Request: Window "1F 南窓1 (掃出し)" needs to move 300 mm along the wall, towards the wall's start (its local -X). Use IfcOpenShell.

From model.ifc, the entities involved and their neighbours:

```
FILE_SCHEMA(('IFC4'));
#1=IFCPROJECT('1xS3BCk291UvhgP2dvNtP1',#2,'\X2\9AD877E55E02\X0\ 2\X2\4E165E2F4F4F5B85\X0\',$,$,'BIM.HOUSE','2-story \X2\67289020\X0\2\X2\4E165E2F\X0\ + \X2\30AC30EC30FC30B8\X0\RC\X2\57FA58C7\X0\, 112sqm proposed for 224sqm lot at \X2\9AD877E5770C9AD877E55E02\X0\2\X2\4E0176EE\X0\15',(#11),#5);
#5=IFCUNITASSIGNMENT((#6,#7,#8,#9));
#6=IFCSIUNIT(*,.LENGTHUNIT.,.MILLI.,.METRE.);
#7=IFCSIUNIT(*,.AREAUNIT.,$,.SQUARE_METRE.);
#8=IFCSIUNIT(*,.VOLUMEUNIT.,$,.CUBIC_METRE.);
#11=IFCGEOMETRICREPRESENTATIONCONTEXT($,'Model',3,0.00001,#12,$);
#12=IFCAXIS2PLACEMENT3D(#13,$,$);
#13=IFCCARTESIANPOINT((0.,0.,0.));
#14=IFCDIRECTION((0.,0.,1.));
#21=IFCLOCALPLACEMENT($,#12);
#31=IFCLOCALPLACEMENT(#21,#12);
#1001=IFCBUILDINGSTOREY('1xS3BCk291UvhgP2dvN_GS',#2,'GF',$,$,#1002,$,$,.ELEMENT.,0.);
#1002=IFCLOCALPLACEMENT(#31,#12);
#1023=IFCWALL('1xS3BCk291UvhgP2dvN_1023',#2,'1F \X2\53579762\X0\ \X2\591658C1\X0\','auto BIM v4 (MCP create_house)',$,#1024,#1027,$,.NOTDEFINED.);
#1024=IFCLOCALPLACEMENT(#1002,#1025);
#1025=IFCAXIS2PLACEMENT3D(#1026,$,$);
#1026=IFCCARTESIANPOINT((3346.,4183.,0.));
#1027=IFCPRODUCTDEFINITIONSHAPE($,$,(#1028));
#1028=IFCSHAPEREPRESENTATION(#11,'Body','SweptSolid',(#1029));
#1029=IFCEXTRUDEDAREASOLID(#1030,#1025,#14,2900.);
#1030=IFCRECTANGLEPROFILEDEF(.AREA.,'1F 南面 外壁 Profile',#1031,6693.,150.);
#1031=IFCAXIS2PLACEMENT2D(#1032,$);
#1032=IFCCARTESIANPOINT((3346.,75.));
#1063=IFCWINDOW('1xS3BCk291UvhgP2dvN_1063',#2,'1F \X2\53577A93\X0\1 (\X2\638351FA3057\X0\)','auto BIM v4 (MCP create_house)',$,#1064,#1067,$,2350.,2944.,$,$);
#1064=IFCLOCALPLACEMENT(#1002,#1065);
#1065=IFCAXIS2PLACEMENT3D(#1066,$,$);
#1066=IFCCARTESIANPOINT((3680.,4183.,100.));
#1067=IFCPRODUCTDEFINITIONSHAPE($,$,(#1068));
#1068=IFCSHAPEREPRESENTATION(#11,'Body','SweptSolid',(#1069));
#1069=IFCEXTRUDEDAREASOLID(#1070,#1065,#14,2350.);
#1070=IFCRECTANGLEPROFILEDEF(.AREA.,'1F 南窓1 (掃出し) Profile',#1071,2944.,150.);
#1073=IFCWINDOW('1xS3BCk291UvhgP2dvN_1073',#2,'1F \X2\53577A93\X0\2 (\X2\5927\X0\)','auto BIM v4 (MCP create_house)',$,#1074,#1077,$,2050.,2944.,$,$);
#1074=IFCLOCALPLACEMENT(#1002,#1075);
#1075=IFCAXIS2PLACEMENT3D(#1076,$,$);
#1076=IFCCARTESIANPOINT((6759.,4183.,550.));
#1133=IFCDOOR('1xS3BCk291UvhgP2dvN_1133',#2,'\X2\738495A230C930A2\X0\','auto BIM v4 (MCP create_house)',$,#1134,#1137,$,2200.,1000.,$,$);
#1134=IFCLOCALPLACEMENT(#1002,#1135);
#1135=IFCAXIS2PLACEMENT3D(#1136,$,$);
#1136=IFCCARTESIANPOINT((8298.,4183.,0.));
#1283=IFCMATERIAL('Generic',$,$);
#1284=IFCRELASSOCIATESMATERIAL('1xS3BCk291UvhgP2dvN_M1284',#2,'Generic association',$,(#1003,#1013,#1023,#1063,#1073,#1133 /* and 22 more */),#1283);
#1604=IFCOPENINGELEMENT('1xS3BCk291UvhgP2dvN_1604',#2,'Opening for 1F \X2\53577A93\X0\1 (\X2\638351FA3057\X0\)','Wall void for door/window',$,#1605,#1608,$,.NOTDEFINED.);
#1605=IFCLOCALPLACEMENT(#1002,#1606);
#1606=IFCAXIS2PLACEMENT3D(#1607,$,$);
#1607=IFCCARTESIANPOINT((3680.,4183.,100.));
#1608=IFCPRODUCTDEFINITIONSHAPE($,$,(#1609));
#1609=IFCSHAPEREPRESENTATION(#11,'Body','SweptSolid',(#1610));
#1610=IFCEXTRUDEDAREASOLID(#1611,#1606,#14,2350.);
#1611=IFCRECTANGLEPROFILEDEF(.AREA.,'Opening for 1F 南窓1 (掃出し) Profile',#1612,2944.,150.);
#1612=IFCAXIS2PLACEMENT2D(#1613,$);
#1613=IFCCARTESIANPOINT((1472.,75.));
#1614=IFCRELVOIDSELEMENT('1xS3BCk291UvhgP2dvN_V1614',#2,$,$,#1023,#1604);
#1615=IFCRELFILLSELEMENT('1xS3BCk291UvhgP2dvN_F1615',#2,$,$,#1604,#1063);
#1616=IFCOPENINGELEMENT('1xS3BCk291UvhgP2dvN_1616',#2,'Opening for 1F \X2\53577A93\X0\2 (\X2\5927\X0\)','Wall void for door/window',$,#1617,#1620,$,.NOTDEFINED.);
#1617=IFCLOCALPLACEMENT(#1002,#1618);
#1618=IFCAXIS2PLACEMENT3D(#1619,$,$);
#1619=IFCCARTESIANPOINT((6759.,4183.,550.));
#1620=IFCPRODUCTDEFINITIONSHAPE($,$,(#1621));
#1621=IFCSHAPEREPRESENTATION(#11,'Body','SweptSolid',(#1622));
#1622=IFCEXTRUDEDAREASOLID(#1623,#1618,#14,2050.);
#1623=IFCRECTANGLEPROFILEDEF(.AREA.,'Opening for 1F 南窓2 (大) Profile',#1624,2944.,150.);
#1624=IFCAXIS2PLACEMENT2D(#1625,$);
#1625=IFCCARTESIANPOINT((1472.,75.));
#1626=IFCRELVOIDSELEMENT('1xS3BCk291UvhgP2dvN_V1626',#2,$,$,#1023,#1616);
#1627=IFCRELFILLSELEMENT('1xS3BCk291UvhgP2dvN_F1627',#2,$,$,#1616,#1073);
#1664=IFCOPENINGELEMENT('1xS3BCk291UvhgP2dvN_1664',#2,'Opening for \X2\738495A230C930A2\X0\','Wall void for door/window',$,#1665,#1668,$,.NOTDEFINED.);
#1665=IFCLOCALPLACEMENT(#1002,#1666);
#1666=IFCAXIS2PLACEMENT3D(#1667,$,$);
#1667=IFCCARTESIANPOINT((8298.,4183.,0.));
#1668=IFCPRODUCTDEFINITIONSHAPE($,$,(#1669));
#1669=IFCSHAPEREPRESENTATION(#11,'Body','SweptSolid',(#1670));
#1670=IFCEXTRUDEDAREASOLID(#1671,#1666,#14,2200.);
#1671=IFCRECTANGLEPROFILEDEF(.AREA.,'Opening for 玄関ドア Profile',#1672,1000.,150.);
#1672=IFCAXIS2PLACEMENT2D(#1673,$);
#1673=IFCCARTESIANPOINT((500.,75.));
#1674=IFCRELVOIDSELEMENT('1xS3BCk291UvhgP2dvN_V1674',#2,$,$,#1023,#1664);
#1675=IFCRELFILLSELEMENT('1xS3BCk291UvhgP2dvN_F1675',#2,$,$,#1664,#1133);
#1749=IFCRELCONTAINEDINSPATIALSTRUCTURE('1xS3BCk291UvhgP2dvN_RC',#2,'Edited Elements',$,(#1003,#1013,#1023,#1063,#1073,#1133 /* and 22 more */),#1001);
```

```python
import ifcopenshell
import ifcopenshell.api.geometry
import ifcopenshell.util.placement
import ifcopenshell.util.unit

model = ifcopenshell.open("model.ifc")
unit_scale = ifcopenshell.util.unit.calculate_unit_scale(model)

window = model.by_guid("1xS3BCk291UvhgP2dvN_1063")
opening = window.FillsVoids[0].RelatingOpeningElement
wall = opening.VoidsElements[0].RelatingBuildingElement

wall_matrix = ifcopenshell.util.placement.get_local_placement(wall.ObjectPlacement)
shift = wall_matrix[:3, 0] * -0.3 / unit_scale
before = ifcopenshell.util.placement.get_local_placement(window.ObjectPlacement)[:3, 3].copy()

# The window is not placed relative to its opening, so move both.
for product in (opening, window):
    matrix = ifcopenshell.util.placement.get_local_placement(product.ObjectPlacement)
    matrix[:3, 3] += shift
    ifcopenshell.api.geometry.edit_object_placement(model, product=product, matrix=matrix, is_si=False)

after = ifcopenshell.util.placement.get_local_placement(window.ObjectPlacement)[:3, 3]
print("window moved by", (after - before).round(3) + 0.0)

model.write("model_rev.ifc")
```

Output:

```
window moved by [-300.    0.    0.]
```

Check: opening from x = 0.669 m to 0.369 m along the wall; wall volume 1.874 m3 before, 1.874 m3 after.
